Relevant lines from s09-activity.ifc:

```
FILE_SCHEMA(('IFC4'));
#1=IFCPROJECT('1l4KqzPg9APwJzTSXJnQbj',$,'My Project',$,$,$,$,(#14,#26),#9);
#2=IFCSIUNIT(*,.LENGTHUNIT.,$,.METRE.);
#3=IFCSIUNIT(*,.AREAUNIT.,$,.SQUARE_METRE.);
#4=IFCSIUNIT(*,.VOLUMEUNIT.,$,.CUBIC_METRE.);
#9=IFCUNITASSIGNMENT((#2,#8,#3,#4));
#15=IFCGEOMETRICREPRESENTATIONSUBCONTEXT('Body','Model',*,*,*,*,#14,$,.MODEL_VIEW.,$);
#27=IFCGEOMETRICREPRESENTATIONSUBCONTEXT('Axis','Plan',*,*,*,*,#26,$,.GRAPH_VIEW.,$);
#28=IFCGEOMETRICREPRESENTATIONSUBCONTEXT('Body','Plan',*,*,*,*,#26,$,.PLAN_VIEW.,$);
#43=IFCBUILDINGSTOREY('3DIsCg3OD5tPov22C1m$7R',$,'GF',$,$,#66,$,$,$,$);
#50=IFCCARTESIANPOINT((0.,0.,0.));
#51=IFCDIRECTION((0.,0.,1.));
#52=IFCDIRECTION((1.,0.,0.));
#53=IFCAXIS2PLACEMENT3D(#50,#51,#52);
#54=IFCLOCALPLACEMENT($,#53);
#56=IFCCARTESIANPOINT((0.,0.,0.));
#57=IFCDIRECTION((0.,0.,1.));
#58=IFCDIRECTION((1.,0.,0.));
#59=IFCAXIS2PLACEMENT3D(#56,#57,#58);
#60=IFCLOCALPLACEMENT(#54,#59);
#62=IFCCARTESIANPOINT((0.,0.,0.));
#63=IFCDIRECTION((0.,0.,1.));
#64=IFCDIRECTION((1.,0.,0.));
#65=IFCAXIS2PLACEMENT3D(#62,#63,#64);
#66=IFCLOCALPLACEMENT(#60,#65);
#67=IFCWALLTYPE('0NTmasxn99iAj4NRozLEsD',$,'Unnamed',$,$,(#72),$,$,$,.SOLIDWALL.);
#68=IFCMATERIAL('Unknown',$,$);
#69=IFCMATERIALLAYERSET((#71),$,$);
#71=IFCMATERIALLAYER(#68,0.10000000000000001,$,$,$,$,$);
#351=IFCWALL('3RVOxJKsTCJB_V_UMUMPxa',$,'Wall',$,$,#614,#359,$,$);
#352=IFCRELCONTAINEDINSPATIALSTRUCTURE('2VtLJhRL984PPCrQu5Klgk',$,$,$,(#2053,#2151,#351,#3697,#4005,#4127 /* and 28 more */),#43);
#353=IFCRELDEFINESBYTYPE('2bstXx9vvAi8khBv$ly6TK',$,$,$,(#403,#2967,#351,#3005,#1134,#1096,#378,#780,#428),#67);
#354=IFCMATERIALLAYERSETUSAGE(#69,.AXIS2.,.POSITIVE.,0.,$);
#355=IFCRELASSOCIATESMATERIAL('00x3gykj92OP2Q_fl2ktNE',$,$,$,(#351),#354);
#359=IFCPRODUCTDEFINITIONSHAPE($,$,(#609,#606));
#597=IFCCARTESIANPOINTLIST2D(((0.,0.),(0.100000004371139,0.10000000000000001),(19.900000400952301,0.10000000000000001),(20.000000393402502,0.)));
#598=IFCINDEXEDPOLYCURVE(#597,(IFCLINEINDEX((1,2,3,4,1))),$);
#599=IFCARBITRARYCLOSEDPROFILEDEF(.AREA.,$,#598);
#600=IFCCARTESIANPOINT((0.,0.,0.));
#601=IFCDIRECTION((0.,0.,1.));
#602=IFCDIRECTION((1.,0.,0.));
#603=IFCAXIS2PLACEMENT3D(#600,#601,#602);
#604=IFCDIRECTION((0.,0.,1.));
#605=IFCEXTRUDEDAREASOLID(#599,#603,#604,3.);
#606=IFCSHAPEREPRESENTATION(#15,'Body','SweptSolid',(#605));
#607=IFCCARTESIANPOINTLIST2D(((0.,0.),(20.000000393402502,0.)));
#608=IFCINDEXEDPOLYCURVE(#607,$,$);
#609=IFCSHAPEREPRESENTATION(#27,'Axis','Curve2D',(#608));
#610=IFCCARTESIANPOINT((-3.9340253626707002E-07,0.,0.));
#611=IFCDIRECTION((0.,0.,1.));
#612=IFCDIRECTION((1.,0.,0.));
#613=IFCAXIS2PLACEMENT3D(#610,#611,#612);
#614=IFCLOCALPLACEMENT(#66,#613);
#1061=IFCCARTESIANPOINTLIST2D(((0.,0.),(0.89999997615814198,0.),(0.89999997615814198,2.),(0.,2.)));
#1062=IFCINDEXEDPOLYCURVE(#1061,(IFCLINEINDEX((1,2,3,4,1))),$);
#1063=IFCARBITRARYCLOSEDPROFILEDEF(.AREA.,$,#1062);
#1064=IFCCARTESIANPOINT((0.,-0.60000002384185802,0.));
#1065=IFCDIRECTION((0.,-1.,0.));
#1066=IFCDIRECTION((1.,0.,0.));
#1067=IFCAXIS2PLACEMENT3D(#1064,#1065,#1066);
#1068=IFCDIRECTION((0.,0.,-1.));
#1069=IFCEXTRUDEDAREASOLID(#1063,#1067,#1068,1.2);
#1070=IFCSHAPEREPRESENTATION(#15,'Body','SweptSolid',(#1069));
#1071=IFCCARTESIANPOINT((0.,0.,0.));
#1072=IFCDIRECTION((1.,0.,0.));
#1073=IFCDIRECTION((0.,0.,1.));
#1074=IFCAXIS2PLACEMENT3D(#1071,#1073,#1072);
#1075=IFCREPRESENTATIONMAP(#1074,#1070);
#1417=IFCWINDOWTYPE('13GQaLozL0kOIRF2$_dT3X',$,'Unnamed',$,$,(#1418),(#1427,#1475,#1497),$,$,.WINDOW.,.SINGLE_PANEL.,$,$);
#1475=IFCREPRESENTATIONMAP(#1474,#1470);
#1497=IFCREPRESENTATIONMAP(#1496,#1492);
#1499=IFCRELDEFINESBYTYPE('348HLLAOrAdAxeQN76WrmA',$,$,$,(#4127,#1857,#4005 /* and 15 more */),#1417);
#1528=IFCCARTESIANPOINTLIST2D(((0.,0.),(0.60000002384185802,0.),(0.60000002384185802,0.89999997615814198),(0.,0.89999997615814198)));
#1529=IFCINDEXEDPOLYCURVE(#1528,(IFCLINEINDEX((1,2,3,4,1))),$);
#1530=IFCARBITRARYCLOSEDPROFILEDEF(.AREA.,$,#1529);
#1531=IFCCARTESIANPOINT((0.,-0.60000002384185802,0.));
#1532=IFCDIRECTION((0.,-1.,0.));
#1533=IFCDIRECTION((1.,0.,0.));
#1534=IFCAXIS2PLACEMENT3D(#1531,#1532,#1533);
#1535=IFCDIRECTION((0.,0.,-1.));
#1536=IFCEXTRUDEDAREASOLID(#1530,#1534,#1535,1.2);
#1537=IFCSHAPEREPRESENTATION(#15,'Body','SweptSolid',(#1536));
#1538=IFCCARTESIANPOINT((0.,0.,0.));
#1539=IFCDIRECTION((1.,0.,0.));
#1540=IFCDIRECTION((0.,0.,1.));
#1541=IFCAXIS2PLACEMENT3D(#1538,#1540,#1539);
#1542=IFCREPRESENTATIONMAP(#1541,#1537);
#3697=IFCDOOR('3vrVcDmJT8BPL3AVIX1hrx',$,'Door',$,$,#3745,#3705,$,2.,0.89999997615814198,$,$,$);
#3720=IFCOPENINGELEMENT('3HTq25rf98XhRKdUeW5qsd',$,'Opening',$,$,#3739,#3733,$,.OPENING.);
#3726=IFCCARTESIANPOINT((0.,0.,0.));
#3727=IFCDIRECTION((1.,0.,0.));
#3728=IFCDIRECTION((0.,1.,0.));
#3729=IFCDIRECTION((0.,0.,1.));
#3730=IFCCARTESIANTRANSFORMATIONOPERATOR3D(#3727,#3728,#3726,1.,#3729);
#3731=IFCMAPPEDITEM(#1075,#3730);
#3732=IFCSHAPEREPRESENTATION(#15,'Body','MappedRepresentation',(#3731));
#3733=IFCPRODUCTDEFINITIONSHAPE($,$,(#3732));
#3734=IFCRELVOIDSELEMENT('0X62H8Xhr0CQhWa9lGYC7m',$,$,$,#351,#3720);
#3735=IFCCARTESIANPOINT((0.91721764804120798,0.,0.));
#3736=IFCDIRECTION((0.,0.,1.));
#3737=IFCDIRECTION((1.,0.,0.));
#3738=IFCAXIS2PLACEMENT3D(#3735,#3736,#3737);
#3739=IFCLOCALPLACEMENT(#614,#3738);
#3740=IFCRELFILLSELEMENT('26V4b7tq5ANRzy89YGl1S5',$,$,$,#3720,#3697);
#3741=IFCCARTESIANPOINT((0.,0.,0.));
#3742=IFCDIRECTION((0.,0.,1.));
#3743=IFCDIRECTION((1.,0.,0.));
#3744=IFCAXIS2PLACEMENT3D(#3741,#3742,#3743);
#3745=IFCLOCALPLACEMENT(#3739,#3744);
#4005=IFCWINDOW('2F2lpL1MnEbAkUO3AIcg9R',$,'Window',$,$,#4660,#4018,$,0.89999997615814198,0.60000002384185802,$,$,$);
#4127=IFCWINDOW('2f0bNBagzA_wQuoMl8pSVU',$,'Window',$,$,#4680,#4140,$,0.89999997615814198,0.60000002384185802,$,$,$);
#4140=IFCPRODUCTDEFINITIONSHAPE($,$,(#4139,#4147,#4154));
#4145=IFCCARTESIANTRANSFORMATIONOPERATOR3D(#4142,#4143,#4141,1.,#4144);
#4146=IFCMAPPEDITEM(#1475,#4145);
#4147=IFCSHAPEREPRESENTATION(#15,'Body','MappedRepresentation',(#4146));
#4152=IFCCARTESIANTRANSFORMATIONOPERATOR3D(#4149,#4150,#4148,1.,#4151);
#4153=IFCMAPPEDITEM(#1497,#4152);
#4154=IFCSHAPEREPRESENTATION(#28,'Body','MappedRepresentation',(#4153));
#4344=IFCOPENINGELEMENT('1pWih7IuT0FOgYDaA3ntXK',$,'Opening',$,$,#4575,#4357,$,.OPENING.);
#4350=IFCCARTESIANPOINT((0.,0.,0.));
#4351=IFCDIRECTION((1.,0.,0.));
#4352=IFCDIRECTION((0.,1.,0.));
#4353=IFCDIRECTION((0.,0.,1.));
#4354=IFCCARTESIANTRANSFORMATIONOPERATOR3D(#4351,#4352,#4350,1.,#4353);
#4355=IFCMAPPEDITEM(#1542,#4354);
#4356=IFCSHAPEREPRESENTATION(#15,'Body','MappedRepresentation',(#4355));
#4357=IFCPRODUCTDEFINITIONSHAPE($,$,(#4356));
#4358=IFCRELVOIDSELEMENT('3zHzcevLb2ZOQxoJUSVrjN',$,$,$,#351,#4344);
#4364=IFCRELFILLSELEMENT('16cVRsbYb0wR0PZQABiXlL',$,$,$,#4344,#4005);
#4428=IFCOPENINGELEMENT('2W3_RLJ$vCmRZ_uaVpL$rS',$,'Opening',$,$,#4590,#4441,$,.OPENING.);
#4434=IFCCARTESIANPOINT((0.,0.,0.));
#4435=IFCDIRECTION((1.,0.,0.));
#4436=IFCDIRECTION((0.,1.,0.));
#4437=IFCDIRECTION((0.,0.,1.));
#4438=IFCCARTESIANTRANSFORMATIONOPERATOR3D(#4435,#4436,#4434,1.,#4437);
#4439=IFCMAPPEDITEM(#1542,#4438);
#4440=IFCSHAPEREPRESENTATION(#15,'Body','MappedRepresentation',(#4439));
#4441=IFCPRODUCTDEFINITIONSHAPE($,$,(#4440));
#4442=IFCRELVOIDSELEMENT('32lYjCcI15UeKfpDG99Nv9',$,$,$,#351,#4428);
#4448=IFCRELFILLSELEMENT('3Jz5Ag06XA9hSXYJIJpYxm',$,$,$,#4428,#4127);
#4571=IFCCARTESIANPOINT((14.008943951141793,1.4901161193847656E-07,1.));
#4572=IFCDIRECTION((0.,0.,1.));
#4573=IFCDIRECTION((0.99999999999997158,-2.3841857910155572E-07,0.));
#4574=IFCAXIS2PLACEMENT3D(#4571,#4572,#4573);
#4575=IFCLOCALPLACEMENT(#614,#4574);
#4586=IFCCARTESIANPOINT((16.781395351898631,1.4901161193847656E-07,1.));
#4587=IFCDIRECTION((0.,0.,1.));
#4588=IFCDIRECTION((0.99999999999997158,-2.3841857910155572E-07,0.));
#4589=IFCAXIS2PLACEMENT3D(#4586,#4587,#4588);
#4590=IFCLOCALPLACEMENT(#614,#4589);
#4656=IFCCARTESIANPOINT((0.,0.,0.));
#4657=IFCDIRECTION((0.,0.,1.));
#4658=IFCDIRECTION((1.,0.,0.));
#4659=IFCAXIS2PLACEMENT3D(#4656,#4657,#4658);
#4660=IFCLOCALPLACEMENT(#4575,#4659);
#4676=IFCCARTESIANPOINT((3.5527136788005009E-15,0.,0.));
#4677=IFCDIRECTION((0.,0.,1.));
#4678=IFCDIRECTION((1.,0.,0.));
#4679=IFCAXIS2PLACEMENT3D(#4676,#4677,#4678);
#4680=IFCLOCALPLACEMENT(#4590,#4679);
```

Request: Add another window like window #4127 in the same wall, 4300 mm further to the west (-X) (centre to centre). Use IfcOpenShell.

```python
import ifcopenshell
import ifcopenshell.api.feature
import ifcopenshell.api.geometry
import ifcopenshell.api.root
import ifcopenshell.geom
import ifcopenshell.util.element
import ifcopenshell.util.placement
import ifcopenshell.util.shape
import ifcopenshell.util.unit

model = ifcopenshell.open("s09-activity.ifc")
unit_scale = ifcopenshell.util.unit.calculate_unit_scale(model)
settings = ifcopenshell.geom.settings()


def volume(element):
    """Net volume in cubic metres, openings subtracted."""
    shape = ifcopenshell.geom.create_shape(settings, element)
    return ifcopenshell.util.shape.get_volume(shape.geometry)


window = model.by_guid("2f0bNBagzA_wQuoMl8pSVU")
opening = window.FillsVoids[0].RelatingOpeningElement
wall = opening.VoidsElements[0].RelatingBuildingElement
before = volume(wall)
shift = ifcopenshell.util.placement.get_local_placement(wall.ObjectPlacement)[:3, 0] * -4.3 / unit_scale

# copy_class copies the void relationship, type, container and properties, but no geometry.
new_opening = ifcopenshell.api.root.copy_class(model, product=opening)
new_opening.Representation = ifcopenshell.util.element.copy_deep(
    model, opening.Representation, exclude=["IfcGeometricRepresentationContext", "IfcRepresentationMap"]
)
new_window = ifcopenshell.api.root.copy_class(model, product=window)
new_window.Representation = ifcopenshell.util.element.copy_deep(
    model, window.Representation, exclude=["IfcGeometricRepresentationContext", "IfcRepresentationMap"]
)
ifcopenshell.api.feature.add_filling(model, opening=new_opening, element=new_window)

for old, new in ((opening, new_opening), (window, new_window)):
    matrix = ifcopenshell.util.placement.get_local_placement(old.ObjectPlacement)
    matrix[:3, 3] += shift
    ifcopenshell.api.geometry.edit_object_placement(model, product=new, matrix=matrix, is_si=False)

after = volume(wall)

print(f"wall volume {before:.3f} -> {after:.3f} m3")

model.write("s09-activity_rev.ifc")
```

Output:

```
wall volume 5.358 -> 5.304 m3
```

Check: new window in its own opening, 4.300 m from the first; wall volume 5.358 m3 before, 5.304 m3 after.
